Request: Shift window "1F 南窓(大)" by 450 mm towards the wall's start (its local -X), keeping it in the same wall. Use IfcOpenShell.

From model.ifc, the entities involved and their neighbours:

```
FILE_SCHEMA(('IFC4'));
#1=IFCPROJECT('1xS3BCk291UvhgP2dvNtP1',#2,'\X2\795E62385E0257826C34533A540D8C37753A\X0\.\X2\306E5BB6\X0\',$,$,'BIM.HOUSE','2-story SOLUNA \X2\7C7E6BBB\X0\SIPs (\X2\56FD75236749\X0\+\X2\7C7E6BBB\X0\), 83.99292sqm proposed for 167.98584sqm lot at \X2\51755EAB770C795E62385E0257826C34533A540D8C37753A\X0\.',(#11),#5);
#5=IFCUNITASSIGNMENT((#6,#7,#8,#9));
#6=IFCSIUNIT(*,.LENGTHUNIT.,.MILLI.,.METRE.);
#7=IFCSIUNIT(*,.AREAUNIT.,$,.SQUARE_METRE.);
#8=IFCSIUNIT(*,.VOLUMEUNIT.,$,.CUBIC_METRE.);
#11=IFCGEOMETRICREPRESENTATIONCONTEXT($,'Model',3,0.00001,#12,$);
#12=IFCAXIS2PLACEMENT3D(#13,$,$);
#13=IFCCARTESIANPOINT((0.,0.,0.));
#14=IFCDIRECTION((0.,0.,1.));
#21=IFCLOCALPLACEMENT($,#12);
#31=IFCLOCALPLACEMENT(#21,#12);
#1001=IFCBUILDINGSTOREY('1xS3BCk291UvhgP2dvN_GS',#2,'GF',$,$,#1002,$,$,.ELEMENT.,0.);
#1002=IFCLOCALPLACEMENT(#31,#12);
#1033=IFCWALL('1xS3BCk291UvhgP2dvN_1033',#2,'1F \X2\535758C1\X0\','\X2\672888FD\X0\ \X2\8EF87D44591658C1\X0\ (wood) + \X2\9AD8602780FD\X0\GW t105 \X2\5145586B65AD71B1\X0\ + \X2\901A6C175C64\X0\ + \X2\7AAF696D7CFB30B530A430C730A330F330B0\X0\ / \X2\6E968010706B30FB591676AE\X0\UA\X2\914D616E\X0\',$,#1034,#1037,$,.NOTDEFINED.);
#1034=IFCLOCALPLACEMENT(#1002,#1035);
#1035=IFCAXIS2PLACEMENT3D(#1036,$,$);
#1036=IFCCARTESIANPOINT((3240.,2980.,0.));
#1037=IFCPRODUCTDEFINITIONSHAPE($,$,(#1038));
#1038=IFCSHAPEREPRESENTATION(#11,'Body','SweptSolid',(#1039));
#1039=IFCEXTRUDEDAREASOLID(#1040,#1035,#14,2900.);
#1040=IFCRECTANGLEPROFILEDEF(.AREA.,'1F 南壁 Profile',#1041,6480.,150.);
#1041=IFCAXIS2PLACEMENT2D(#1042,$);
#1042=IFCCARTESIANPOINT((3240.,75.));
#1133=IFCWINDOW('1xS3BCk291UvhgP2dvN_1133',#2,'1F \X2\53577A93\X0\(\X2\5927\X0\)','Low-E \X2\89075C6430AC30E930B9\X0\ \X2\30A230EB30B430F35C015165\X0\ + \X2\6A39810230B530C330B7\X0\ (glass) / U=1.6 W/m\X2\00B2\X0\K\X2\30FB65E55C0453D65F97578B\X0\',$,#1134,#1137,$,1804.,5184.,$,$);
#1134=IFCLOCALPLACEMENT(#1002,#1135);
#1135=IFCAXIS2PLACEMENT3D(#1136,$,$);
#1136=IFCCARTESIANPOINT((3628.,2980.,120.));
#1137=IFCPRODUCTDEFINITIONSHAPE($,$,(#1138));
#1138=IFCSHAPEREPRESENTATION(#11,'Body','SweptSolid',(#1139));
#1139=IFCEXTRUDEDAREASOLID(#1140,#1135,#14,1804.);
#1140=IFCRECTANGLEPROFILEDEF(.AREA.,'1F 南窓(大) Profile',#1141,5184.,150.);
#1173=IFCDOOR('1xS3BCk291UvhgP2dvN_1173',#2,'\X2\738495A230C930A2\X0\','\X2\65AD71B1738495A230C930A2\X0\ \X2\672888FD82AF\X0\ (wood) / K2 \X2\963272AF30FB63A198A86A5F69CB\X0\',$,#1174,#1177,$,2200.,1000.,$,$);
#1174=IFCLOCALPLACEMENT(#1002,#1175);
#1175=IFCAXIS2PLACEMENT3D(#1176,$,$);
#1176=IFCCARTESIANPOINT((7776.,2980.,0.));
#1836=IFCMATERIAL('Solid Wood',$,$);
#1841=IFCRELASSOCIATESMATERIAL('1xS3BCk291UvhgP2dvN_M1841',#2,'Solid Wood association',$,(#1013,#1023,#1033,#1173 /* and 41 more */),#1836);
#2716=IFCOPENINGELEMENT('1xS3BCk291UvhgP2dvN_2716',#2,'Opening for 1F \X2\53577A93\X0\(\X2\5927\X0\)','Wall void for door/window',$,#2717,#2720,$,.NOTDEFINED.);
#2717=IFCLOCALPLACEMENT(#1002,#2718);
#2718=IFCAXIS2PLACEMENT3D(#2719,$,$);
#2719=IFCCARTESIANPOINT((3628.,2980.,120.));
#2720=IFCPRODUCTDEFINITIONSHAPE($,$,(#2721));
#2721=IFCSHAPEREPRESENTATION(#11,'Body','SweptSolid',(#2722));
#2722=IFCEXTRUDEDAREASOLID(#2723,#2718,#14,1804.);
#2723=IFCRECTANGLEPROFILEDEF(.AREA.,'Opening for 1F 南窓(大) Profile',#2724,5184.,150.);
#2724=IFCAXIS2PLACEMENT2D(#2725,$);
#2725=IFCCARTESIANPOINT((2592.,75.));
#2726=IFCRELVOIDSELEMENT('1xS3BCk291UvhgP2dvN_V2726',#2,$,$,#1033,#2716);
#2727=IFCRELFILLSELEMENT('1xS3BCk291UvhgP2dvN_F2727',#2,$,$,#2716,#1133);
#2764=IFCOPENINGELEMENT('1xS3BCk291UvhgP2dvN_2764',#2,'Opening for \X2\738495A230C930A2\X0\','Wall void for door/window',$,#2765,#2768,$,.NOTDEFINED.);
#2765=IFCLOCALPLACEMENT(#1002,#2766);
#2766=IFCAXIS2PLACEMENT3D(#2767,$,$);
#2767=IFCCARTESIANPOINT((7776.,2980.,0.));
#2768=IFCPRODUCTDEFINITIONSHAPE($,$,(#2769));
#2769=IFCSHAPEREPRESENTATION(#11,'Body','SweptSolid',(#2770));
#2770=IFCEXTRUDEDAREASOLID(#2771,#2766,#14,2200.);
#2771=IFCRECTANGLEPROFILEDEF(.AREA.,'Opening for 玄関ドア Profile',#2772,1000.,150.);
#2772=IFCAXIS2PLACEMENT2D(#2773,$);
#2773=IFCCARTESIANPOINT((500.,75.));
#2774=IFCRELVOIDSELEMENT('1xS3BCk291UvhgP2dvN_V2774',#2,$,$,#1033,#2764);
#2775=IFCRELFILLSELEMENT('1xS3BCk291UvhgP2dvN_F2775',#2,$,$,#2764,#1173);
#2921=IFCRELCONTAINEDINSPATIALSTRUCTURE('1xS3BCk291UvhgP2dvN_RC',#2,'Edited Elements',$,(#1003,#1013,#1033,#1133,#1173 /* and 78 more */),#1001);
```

```python
import ifcopenshell
import ifcopenshell.api.geometry
import ifcopenshell.util.placement

model = ifcopenshell.open("model.ifc")

window = model.by_id(1133)
opening = window.FillsVoids[0].RelatingOpeningElement
wall = opening.VoidsElements[0].RelatingBuildingElement

wall_matrix = ifcopenshell.util.placement.get_local_placement(wall.ObjectPlacement)
shift = wall_matrix[:3, 0] * -450.0
before = ifcopenshell.util.placement.get_local_placement(window.ObjectPlacement)[:3, 3].copy()

# The window is not placed relative to its opening, so move both.
for product in (opening, window):
    matrix = ifcopenshell.util.placement.get_local_placement(product.ObjectPlacement)
    matrix[:3, 3] += shift
    ifcopenshell.api.geometry.edit_object_placement(model, product=product, matrix=matrix, is_si=False)

after = ifcopenshell.util.placement.get_local_placement(window.ObjectPlacement)[:3, 3]
print("window moved by", (after - before).round(3) + 0.0)

model.write("model-out.ifc")
```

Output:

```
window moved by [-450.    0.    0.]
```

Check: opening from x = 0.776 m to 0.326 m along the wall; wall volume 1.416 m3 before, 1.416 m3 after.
